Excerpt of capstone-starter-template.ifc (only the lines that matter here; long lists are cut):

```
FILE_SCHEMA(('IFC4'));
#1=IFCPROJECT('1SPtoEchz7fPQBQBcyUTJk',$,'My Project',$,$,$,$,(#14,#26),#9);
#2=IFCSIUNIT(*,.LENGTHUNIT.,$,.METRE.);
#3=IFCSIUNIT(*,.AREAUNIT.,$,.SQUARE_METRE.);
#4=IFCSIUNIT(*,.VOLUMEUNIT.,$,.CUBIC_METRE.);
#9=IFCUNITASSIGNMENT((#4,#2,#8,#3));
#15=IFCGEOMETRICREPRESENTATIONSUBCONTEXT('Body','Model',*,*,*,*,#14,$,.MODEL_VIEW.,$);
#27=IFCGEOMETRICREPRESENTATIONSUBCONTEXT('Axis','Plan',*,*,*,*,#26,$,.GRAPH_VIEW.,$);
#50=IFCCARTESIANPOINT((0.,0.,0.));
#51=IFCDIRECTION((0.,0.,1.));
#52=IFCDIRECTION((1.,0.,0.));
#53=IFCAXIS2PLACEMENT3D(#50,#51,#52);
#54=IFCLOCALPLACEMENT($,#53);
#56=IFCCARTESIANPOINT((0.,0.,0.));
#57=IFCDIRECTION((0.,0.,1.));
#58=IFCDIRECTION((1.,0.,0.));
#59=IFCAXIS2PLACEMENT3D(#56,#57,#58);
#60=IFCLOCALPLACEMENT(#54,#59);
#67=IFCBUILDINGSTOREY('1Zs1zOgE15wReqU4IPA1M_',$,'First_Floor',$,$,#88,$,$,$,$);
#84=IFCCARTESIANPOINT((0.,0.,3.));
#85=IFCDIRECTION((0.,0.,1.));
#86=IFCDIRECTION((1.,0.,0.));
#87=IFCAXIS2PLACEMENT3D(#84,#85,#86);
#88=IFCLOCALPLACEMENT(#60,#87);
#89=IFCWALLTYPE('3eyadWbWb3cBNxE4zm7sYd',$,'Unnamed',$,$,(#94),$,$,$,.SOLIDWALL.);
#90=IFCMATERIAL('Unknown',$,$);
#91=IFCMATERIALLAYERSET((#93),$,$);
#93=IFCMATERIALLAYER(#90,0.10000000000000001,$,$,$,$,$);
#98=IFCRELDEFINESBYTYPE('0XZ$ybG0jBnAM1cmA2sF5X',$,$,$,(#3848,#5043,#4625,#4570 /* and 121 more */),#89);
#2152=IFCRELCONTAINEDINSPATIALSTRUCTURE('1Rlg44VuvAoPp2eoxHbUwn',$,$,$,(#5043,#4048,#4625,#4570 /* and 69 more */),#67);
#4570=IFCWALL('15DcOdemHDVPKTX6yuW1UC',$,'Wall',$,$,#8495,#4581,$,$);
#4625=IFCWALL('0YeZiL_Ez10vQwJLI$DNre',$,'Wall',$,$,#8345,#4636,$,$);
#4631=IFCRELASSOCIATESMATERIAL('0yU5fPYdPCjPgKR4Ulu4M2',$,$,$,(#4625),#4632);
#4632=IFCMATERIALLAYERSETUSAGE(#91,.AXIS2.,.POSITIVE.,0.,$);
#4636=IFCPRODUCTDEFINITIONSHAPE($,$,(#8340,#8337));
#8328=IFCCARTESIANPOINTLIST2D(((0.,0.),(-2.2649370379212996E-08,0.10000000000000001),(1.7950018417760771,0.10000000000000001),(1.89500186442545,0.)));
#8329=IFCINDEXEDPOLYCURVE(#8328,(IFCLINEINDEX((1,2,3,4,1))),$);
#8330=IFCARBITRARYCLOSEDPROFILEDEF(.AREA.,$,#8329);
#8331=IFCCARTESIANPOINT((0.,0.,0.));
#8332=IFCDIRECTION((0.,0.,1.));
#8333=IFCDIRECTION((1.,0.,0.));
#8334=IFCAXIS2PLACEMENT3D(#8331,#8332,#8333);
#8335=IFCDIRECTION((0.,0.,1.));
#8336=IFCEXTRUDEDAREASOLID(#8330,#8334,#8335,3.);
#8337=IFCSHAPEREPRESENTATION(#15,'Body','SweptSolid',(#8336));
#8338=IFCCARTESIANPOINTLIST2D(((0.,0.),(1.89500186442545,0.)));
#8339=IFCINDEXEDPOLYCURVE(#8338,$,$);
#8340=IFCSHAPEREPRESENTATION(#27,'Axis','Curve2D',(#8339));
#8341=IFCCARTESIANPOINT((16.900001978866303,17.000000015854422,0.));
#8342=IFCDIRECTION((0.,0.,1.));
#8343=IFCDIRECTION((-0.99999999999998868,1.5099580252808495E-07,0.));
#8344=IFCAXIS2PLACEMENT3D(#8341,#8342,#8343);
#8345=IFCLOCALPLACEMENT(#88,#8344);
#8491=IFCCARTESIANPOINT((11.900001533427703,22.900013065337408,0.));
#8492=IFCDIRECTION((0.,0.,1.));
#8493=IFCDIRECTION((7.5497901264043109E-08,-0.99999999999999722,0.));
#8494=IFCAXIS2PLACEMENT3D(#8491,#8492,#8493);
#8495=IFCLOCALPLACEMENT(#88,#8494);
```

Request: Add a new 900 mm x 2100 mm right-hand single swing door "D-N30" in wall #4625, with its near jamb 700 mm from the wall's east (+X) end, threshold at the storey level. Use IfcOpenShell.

```python
import numpy as np
import ifcopenshell
import ifcopenshell.api.feature
import ifcopenshell.api.geometry
import ifcopenshell.api.root
import ifcopenshell.api.spatial
import ifcopenshell.geom
import ifcopenshell.util.element
import ifcopenshell.util.placement
import ifcopenshell.util.representation
import ifcopenshell.util.shape
import ifcopenshell.util.unit

model = ifcopenshell.open("capstone-starter-template.ifc")
unit_scale = ifcopenshell.util.unit.calculate_unit_scale(model)
settings = ifcopenshell.geom.settings()


def volume(element):
    """Net volume in cubic metres, openings subtracted."""
    shape = ifcopenshell.geom.create_shape(settings, element)
    return ifcopenshell.util.shape.get_volume(shape.geometry)


wall = model.by_id(4625)
storey = ifcopenshell.util.element.get_container(wall, ifc_class="IfcBuildingStorey")
context = ifcopenshell.util.representation.get_context(model, "Model", "Body", "MODEL_VIEW")
before = volume(wall)

width, height, from_end, sill = 0.9, 2.1, 0.7, 0.0  # metres

# The wall runs along its own X axis, and the end named is its -X end.
wall_shape = ifcopenshell.geom.create_shape(settings, wall)
x, y, z = ifcopenshell.util.shape.get_vertices(wall_shape.geometry).T
start = x.min() + from_end
face, thickness = float(y.min()), float(y.max() - y.min())
wall_matrix = ifcopenshell.util.placement.get_local_placement(wall.ObjectPlacement)
level = ifcopenshell.util.placement.get_local_placement(storey.ObjectPlacement)[2, 3]


def in_wall(x, y):
    """Placement at x, y metres in the wall's axes, at sill height."""
    matrix = wall_matrix.copy()
    matrix[:, 3] = wall_matrix @ np.array([x / unit_scale, y / unit_scale, 0.0, 1.0])
    matrix[2, 3] = level + sill / unit_scale
    return matrix


# Opening: a box that overshoots both wall faces by 50 mm.
opening = ifcopenshell.api.root.create_entity(model, ifc_class="IfcOpeningElement", predefined_type="OPENING")
box = ifcopenshell.api.geometry.add_wall_representation(
    model, context=context, length=width, height=height, thickness=thickness + 0.1
)
ifcopenshell.api.geometry.assign_representation(model, product=opening, representation=box)
ifcopenshell.api.geometry.edit_object_placement(model, product=opening, matrix=in_wall(start, face - 0.05), is_si=False)
ifcopenshell.api.feature.add_feature(model, feature=opening, element=wall)

door = ifcopenshell.api.root.create_entity(model, ifc_class="IfcDoor", name="D-N30", predefined_type="DOOR")
door.OverallWidth, door.OverallHeight = width / unit_scale, height / unit_scale
door.OperationType = "SINGLE_SWING_RIGHT"
body = ifcopenshell.api.geometry.add_door_representation(
    model,
    context=context,
    overall_width=door.OverallWidth,
    overall_height=door.OverallHeight,
    operation_type="SINGLE_SWING_RIGHT",
    lining_properties={"LiningDepth": thickness / unit_scale, "ThresholdDepth": thickness / unit_scale},
)
ifcopenshell.api.geometry.assign_representation(model, product=door, representation=body)
ifcopenshell.api.spatial.assign_container(model, products=[door], relating_structure=storey)
ifcopenshell.api.feature.add_filling(model, opening=opening, element=door)

# The lining spans the wall, so the door starts at the wall face.
ifcopenshell.api.geometry.edit_object_placement(model, product=door, matrix=in_wall(start, face), is_si=False)

after = volume(wall)

print(f"wall volume {before:.3f} -> {after:.3f} m3")

model.write("capstone-starter-template_updated.ifc")
```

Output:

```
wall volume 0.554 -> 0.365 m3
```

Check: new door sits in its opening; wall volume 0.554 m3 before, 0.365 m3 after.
